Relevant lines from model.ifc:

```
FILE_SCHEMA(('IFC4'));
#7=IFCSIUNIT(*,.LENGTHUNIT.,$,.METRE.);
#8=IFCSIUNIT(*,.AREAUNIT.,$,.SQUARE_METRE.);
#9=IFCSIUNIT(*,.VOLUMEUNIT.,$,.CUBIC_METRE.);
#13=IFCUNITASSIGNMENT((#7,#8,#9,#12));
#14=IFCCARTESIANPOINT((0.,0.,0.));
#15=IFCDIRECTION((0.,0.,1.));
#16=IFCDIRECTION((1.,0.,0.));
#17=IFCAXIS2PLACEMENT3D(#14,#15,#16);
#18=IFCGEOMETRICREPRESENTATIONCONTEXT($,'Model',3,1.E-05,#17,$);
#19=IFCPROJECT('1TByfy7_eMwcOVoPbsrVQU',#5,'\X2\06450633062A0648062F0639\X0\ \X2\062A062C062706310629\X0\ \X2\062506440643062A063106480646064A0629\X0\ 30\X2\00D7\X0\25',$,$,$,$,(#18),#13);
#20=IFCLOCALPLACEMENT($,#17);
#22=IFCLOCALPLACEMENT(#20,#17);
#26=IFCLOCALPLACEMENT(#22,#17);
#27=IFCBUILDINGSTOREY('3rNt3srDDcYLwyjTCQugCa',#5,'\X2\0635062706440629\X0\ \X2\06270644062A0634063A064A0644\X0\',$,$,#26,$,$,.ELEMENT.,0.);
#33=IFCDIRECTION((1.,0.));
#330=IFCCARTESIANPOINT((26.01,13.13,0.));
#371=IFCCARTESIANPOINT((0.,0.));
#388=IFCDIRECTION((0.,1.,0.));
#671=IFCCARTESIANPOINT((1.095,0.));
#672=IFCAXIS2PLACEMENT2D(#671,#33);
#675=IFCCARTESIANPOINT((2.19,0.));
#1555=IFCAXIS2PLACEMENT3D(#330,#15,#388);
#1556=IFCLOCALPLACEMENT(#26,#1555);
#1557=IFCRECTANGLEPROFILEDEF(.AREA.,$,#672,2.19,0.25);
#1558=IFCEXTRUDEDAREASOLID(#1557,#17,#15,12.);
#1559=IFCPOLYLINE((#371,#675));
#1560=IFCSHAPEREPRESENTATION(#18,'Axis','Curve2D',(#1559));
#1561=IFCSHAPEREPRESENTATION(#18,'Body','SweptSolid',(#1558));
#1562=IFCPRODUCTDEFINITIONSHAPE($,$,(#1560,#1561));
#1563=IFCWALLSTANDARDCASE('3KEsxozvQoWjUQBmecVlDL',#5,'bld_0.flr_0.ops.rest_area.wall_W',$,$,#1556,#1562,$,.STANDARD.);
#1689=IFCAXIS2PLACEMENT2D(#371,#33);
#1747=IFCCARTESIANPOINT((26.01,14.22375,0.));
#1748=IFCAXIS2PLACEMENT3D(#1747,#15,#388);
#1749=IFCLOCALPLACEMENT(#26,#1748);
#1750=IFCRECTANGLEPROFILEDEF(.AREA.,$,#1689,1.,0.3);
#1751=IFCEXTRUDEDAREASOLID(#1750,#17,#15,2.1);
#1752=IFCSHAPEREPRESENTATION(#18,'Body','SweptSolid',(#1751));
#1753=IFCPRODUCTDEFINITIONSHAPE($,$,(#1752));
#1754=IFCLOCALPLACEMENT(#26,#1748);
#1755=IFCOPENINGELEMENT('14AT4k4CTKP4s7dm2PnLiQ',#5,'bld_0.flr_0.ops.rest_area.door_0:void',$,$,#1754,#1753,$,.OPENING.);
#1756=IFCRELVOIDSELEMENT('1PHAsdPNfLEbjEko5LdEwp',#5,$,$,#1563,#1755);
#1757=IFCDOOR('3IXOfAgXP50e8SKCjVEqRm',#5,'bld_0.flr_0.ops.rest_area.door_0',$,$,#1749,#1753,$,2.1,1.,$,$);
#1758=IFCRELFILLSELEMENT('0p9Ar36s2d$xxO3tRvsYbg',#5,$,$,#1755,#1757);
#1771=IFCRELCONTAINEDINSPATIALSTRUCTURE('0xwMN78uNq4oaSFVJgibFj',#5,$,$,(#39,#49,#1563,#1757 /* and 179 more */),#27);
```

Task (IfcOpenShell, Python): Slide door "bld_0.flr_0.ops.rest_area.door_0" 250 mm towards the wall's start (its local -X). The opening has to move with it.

```python
import ifcopenshell
import ifcopenshell.api.geometry
import ifcopenshell.util.placement
import ifcopenshell.util.unit

model = ifcopenshell.open("model.ifc")
unit_scale = ifcopenshell.util.unit.calculate_unit_scale(model)

door = model.by_guid("3IXOfAgXP50e8SKCjVEqRm")
opening = door.FillsVoids[0].RelatingOpeningElement
wall = opening.VoidsElements[0].RelatingBuildingElement

wall_matrix = ifcopenshell.util.placement.get_local_placement(wall.ObjectPlacement)
shift = wall_matrix[:3, 0] * -0.25 / unit_scale
before = ifcopenshell.util.placement.get_local_placement(door.ObjectPlacement)[:3, 3].copy()

# The door is not placed relative to its opening, so move both.
for product in (opening, door):
    matrix = ifcopenshell.util.placement.get_local_placement(product.ObjectPlacement)
    matrix[:3, 3] += shift
    ifcopenshell.api.geometry.edit_object_placement(model, product=product, matrix=matrix, is_si=False)

after = ifcopenshell.util.placement.get_local_placement(door.ObjectPlacement)[:3, 3]
print("door moved by", (after - before).round(3) + 0.0)

model.write("model_edited.ifc")
```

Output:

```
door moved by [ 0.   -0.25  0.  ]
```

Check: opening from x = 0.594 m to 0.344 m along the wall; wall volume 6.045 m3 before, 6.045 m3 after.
